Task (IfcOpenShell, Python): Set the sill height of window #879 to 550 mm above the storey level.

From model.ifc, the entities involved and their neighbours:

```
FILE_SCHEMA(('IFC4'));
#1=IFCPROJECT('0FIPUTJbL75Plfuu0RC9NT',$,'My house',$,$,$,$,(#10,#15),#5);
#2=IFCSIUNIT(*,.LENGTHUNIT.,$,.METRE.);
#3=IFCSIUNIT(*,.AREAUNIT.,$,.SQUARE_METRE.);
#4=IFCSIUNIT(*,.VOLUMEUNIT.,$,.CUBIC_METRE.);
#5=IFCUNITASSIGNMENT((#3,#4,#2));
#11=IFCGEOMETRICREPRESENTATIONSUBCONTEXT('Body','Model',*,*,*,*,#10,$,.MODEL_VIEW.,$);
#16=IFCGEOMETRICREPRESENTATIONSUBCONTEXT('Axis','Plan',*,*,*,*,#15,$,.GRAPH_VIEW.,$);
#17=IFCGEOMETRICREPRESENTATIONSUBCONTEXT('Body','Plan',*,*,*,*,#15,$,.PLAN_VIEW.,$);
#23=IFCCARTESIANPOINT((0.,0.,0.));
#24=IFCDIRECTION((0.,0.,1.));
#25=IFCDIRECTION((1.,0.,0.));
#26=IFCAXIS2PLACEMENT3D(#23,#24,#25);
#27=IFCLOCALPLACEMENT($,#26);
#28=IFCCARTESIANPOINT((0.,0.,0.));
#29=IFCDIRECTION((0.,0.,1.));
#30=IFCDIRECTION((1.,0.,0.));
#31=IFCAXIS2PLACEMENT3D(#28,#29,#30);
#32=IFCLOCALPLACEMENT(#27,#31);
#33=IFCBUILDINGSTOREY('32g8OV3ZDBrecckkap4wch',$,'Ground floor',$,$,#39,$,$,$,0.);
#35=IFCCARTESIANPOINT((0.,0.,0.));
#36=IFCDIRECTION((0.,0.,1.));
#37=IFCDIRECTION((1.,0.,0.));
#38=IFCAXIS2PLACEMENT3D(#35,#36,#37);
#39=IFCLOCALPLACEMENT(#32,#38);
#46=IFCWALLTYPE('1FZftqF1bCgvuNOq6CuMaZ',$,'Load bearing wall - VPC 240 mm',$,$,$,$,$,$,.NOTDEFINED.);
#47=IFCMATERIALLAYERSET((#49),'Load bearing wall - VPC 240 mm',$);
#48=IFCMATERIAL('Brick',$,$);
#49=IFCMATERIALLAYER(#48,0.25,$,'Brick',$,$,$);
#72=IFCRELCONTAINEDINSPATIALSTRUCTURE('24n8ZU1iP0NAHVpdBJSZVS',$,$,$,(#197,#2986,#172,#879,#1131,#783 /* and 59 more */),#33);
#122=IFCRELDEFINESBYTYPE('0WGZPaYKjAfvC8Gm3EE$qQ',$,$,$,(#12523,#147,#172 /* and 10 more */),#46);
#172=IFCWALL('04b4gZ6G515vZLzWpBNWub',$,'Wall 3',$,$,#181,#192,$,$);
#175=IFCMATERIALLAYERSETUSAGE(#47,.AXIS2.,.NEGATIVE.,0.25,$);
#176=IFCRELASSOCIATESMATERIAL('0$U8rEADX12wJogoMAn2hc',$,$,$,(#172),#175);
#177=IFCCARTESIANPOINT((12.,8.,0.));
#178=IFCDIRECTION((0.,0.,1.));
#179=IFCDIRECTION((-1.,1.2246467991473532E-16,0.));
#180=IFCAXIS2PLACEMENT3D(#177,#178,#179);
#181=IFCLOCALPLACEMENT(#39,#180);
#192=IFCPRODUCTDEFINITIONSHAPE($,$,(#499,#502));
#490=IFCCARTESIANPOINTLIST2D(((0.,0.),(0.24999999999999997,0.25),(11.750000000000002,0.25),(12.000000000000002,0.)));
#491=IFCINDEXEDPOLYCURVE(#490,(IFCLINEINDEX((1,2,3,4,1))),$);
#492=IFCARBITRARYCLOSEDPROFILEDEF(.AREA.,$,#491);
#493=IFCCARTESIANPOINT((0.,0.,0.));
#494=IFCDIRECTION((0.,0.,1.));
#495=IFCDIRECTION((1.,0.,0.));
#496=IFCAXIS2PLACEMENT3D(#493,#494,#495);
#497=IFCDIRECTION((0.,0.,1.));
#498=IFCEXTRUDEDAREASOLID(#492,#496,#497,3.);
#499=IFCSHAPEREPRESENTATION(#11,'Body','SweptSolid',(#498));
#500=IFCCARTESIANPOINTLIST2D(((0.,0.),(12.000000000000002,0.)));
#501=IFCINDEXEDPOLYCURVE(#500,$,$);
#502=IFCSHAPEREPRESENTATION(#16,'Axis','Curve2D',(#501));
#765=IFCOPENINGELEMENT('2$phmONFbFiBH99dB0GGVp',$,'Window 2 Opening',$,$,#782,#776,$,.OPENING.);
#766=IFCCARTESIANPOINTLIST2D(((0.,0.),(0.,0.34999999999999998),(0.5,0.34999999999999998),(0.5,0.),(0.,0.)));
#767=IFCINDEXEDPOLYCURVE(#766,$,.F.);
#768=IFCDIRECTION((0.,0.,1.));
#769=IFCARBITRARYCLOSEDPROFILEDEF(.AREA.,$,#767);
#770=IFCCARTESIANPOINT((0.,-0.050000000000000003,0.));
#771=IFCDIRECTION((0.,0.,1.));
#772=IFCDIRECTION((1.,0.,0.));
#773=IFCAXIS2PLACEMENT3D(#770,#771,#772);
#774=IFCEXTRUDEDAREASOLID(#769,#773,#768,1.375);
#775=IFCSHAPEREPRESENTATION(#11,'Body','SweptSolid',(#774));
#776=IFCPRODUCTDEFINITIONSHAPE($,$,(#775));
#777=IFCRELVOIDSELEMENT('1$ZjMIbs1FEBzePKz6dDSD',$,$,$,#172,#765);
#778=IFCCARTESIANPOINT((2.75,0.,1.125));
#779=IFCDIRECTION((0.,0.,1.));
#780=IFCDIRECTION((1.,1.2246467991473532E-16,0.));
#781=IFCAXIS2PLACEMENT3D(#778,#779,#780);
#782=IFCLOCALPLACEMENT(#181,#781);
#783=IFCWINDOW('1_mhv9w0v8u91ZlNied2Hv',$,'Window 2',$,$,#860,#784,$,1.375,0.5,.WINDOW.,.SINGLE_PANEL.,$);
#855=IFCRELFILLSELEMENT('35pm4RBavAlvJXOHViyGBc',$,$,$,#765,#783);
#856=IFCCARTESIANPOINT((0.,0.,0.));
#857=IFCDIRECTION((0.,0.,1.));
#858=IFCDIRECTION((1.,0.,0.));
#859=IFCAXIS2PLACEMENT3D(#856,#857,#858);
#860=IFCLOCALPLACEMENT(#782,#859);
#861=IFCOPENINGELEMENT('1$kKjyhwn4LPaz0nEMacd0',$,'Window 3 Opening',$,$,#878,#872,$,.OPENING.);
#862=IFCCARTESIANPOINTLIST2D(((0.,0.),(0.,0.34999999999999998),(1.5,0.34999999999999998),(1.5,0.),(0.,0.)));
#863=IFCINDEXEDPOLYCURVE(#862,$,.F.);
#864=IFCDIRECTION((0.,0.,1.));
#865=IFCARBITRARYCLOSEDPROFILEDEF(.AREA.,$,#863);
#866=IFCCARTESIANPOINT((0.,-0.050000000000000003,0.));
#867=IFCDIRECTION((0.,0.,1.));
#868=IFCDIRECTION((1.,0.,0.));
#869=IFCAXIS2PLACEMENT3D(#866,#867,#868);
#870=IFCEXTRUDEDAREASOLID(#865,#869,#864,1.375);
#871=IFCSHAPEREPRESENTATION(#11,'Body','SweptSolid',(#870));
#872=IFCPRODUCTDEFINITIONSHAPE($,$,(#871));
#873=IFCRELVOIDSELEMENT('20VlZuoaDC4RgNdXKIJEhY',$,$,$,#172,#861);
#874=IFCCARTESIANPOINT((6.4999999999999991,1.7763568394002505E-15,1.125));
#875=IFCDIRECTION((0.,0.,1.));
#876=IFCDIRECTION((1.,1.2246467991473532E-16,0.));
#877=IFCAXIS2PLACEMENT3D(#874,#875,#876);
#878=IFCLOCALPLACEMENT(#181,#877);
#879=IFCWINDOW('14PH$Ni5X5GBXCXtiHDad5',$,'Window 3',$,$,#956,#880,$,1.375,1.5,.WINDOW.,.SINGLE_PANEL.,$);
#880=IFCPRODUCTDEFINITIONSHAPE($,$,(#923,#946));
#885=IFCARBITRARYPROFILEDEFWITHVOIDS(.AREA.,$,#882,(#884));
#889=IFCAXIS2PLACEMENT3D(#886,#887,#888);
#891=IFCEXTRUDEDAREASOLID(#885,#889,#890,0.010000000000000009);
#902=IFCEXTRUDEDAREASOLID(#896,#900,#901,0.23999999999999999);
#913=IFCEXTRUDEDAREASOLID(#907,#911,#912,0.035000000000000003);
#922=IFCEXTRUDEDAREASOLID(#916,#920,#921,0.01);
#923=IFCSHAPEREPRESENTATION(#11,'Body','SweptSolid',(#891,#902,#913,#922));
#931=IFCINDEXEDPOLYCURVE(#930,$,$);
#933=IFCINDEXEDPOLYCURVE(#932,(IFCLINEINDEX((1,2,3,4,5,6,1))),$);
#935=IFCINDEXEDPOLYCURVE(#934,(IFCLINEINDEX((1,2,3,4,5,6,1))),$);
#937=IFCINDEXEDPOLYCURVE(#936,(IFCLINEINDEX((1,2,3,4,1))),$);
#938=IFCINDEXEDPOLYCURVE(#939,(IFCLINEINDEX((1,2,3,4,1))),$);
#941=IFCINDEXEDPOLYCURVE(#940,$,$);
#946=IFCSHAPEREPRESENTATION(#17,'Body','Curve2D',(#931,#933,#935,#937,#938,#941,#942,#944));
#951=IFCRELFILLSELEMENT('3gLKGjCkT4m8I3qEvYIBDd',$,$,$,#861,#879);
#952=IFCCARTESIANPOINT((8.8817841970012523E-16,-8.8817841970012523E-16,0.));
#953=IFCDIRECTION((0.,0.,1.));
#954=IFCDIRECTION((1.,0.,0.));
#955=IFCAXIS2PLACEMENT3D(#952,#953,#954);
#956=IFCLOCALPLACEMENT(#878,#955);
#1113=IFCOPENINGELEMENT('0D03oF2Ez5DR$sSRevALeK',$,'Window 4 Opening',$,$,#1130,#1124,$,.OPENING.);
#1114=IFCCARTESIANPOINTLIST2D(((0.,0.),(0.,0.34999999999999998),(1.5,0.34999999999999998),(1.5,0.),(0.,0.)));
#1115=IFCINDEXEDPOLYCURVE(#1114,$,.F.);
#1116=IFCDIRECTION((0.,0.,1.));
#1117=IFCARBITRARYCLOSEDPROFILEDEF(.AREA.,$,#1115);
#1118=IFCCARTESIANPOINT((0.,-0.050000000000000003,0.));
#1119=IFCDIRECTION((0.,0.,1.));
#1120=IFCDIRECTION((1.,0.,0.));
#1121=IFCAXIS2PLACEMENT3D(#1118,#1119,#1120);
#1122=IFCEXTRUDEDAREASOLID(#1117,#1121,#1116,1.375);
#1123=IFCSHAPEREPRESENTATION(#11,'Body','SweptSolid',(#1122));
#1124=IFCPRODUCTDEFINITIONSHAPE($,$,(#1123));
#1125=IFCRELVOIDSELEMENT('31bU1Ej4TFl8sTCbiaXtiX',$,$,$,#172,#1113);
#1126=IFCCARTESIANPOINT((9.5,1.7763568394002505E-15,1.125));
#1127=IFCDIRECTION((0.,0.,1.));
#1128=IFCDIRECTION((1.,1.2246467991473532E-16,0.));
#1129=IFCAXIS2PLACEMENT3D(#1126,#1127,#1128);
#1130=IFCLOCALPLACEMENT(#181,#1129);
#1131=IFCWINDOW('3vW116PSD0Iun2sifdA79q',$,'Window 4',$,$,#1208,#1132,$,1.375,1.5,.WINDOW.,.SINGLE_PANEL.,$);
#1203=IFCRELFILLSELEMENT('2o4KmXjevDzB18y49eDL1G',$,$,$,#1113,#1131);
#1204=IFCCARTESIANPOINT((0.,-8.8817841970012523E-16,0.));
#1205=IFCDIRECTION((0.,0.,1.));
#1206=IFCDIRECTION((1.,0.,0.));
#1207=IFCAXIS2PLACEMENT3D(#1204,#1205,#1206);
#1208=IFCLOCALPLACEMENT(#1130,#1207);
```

```python
import numpy as np
import ifcopenshell
import ifcopenshell.api.geometry
import ifcopenshell.geom
import ifcopenshell.util.element
import ifcopenshell.util.placement
import ifcopenshell.util.shape
import ifcopenshell.util.unit

model = ifcopenshell.open("model.ifc")
unit_scale = ifcopenshell.util.unit.calculate_unit_scale(model)

window = model.by_guid("14PH$Ni5X5GBXCXtiHDad5")
opening = window.FillsVoids[0].RelatingOpeningElement
storey = ifcopenshell.util.element.get_container(window, ifc_class="IfcBuildingStorey")
level = ifcopenshell.util.placement.get_local_placement(storey.ObjectPlacement)[2, 3]

# The opening's origin need not be at the sill, so measure its lowest point.
shape = ifcopenshell.geom.create_shape(ifcopenshell.geom.settings(), opening)
bottom = ifcopenshell.util.shape.get_shape_bottom_elevation(shape, shape.geometry) / unit_scale
dz = level + 0.55 - bottom

shift = np.array([0.0, 0.0, dz])
# The window is placed relative to its opening, so it follows when the opening moves.
matrix = ifcopenshell.util.placement.get_local_placement(opening.ObjectPlacement)
matrix[:3, 3] += shift
ifcopenshell.api.geometry.edit_object_placement(
    model, product=opening, matrix=matrix, is_si=False, should_transform_children=True
)

print(f"moved by {dz * unit_scale:+.3f} m")

model.write("model_v2.ifc")
```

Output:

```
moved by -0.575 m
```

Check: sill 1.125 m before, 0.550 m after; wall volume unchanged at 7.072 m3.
